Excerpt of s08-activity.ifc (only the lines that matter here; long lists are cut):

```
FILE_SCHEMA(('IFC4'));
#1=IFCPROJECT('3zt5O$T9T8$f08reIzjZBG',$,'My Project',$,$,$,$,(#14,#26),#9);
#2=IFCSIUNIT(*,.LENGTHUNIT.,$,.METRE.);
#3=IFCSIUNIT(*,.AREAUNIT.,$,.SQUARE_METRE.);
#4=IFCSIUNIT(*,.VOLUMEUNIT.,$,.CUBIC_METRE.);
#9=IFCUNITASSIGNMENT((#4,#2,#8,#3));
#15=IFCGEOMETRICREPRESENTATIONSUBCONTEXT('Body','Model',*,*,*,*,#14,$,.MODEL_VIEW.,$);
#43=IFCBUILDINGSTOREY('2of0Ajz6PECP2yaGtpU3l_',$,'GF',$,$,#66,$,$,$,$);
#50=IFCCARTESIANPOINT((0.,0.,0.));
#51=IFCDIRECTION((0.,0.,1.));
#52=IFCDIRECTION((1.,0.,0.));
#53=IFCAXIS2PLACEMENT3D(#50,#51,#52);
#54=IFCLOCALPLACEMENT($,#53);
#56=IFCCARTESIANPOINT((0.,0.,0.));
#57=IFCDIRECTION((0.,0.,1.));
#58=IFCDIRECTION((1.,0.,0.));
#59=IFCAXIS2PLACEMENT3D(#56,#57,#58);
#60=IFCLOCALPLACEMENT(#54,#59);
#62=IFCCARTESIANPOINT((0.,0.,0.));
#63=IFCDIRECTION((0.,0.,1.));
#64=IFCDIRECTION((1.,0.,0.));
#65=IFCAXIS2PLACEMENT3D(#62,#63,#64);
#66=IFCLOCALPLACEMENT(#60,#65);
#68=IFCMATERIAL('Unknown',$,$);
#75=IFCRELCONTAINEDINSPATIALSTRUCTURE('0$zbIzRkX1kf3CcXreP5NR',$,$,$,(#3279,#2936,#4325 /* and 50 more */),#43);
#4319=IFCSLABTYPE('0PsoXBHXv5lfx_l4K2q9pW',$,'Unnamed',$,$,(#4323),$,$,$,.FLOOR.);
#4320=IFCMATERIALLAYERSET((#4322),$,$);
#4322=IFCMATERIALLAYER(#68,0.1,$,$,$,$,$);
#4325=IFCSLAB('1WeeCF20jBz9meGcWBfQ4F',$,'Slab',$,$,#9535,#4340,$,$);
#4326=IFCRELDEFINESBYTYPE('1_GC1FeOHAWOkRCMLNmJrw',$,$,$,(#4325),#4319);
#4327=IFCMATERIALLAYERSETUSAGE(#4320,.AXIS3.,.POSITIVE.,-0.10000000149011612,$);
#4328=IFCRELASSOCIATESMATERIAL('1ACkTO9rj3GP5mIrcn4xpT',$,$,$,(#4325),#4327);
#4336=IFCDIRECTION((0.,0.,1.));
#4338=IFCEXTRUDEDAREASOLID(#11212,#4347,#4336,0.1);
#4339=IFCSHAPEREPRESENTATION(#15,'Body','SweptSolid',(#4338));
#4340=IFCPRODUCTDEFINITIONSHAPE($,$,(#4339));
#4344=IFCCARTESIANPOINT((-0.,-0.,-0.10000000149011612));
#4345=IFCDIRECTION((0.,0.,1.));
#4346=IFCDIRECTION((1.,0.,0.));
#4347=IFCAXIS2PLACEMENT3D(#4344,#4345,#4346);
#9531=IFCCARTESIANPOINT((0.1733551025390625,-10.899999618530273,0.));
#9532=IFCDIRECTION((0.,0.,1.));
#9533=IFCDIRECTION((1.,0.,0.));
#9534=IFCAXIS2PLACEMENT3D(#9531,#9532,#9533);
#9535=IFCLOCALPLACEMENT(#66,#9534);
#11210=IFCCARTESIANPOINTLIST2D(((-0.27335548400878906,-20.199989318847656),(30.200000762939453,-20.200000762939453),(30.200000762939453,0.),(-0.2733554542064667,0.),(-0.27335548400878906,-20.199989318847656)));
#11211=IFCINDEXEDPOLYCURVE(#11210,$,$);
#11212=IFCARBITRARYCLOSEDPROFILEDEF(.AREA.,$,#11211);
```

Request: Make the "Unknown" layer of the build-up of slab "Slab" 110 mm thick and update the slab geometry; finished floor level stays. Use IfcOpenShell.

```python
import ifcopenshell
import ifcopenshell.util.element
import ifcopenshell.util.representation

model = ifcopenshell.open("s08-activity.ifc")

layer_set = model.by_id(4320)
layer = next(l for l in layer_set.MaterialLayers if l.Material and l.Material.Name == "Unknown")
change = 0.11 - layer.LayerThickness
layer.LayerThickness += change

# Geometry does not follow the layer set by itself.
slabs = [e for e in ifcopenshell.util.element.get_elements_by_material(model, layer_set) if e.is_a("IfcSlab")]
for slab in sorted(slabs, key=lambda e: e.id()):
    body = ifcopenshell.util.representation.get_representation(slab, "Model", "Body")
    solid = body.Items[0]
    old_depth = solid.Depth
    solid.Depth += change
    # Extruded upwards: lower the start of the extrusion so the top stays.
    x, y, z = solid.Position.Location.Coordinates
    solid.Position.Location = model.createIfcCartesianPoint((x, y, z - change))
    print(slab.id(), f"{old_depth:g} -> {solid.Depth:g}")

# The layers are counted up from the underside, which has moved.
for usage in {ifcopenshell.util.element.get_material(slab) for slab in slabs}:
    usage.OffsetFromReferenceLine -= change

model.write("s08-activity-out.ifc")
```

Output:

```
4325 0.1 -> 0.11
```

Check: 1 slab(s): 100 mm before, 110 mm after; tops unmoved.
